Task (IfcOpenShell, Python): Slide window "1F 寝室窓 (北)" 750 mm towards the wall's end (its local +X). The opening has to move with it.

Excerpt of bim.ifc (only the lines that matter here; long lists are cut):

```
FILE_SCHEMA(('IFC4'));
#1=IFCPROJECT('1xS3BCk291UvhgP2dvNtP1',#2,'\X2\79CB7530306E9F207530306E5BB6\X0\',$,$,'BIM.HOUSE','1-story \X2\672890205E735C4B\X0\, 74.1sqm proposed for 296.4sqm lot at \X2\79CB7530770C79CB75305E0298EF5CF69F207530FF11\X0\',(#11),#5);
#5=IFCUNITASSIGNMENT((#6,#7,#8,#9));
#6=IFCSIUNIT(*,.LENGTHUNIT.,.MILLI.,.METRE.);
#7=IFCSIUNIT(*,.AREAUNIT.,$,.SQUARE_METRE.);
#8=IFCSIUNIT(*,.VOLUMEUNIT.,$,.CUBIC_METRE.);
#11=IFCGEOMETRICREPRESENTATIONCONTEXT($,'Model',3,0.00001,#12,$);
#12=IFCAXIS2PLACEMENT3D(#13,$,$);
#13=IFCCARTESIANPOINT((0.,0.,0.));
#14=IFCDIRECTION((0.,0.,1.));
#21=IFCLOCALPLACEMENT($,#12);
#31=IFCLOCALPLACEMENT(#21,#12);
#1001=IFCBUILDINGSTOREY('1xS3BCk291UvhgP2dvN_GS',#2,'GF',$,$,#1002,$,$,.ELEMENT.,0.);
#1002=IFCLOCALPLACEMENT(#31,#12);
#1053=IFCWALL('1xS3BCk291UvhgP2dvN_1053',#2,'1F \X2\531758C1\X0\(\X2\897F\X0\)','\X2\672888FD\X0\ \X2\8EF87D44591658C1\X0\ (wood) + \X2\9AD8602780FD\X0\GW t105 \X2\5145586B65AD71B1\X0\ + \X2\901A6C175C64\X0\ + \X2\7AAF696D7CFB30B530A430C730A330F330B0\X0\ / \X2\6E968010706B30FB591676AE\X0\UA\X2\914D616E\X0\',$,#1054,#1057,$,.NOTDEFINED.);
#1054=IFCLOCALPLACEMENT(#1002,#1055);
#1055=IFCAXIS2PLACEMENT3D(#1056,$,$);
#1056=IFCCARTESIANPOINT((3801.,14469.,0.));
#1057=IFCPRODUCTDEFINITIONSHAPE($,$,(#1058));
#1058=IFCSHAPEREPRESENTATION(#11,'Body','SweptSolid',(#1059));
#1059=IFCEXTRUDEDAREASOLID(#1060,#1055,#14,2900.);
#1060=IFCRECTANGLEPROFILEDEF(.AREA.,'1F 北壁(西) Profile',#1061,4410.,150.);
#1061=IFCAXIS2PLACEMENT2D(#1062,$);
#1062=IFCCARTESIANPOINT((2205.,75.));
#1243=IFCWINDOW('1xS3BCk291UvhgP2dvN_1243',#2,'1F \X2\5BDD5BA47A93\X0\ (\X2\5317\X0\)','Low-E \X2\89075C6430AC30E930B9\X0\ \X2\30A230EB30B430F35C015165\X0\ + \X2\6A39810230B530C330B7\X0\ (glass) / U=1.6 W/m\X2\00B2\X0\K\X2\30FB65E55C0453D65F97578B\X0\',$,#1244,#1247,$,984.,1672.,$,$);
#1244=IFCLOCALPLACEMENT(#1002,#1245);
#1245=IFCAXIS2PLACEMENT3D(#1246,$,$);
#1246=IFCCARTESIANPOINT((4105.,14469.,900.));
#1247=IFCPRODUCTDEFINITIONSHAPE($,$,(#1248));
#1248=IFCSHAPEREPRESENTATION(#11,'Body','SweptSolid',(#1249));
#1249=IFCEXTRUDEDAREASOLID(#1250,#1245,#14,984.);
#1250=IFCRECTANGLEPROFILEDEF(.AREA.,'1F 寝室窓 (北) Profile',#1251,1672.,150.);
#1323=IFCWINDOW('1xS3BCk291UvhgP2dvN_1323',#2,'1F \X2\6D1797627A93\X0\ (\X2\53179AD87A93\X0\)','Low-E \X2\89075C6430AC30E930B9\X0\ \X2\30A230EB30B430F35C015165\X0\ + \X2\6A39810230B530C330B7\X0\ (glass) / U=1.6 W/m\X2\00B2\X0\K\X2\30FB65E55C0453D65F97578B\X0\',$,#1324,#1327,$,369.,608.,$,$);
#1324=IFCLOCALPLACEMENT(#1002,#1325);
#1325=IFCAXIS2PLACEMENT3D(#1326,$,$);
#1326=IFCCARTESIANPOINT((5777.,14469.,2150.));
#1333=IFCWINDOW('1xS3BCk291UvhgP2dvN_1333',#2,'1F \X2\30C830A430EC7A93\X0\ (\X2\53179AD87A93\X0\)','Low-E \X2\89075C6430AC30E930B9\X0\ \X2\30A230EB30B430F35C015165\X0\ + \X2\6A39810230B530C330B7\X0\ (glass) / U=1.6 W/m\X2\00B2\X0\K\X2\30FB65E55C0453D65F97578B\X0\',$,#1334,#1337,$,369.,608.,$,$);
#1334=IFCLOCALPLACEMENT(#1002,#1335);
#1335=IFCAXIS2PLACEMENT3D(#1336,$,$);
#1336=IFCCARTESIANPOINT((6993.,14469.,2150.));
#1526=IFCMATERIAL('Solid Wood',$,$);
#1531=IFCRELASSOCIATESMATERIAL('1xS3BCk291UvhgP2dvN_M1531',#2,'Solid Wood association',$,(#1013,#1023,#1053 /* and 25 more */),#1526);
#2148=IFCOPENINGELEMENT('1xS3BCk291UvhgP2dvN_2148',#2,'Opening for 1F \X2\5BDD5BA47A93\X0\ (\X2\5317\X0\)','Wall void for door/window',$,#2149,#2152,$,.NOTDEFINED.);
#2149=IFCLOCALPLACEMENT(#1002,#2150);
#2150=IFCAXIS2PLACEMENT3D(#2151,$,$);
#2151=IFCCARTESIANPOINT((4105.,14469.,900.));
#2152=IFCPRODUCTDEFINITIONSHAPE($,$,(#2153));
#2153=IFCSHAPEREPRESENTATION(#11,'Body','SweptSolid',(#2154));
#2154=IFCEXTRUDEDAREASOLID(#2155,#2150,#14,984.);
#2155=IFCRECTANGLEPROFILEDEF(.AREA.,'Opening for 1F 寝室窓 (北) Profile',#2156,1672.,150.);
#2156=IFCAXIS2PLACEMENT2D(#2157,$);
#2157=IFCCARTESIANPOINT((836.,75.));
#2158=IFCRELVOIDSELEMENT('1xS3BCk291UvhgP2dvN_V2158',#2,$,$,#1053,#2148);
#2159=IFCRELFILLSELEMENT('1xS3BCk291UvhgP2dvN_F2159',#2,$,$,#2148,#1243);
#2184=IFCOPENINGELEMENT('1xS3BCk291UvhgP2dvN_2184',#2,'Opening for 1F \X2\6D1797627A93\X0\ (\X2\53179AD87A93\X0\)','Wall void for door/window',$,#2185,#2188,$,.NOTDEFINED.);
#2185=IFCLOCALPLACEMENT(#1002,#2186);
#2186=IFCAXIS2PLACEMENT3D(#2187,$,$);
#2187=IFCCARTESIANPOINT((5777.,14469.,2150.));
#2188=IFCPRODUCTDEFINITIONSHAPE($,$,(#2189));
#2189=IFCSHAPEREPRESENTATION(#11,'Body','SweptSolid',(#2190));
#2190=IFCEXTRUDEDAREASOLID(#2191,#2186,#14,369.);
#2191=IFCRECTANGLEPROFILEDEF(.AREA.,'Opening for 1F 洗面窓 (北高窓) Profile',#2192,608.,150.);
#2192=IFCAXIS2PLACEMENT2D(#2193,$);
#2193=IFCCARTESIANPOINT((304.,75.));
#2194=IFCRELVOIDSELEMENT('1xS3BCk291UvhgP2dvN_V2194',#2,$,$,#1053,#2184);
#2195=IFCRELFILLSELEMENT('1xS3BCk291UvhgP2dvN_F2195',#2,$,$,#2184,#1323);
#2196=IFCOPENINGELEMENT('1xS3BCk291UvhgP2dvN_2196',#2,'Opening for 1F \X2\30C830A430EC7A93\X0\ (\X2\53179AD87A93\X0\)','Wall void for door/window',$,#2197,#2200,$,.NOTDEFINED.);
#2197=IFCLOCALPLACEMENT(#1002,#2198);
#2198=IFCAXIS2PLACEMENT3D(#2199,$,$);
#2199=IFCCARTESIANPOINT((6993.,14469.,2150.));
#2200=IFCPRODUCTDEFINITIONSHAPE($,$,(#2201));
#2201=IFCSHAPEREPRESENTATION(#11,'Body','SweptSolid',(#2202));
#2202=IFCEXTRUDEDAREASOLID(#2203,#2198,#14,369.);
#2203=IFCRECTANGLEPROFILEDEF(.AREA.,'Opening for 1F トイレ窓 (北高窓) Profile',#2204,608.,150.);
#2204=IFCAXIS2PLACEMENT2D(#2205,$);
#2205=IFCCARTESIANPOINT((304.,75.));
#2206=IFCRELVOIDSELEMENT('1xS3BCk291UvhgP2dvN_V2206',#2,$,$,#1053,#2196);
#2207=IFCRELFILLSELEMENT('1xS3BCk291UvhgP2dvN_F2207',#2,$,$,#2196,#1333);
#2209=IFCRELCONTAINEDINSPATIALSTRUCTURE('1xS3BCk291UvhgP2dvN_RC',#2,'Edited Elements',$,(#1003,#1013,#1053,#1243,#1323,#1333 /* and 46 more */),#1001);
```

```python
import ifcopenshell
import ifcopenshell.api.geometry
import ifcopenshell.util.placement

model = ifcopenshell.open("bim.ifc")

window = model.by_guid("1xS3BCk291UvhgP2dvN_1243")
opening = window.FillsVoids[0].RelatingOpeningElement
wall = opening.VoidsElements[0].RelatingBuildingElement

wall_matrix = ifcopenshell.util.placement.get_local_placement(wall.ObjectPlacement)
shift = wall_matrix[:3, 0] * 750.0
before = ifcopenshell.util.placement.get_local_placement(window.ObjectPlacement)[:3, 3].copy()

# The window is not placed relative to its opening, so move both.
for product in (opening, window):
    matrix = ifcopenshell.util.placement.get_local_placement(product.ObjectPlacement)
    matrix[:3, 3] += shift
    ifcopenshell.api.geometry.edit_object_placement(model, product=product, matrix=matrix, is_si=False)

after = ifcopenshell.util.placement.get_local_placement(window.ObjectPlacement)[:3, 3]
print("window moved by", (after - before).round(3) + 0.0)

model.write("bim_updated.ifc")
```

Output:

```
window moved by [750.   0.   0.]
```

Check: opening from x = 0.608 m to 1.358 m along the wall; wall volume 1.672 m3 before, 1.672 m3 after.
